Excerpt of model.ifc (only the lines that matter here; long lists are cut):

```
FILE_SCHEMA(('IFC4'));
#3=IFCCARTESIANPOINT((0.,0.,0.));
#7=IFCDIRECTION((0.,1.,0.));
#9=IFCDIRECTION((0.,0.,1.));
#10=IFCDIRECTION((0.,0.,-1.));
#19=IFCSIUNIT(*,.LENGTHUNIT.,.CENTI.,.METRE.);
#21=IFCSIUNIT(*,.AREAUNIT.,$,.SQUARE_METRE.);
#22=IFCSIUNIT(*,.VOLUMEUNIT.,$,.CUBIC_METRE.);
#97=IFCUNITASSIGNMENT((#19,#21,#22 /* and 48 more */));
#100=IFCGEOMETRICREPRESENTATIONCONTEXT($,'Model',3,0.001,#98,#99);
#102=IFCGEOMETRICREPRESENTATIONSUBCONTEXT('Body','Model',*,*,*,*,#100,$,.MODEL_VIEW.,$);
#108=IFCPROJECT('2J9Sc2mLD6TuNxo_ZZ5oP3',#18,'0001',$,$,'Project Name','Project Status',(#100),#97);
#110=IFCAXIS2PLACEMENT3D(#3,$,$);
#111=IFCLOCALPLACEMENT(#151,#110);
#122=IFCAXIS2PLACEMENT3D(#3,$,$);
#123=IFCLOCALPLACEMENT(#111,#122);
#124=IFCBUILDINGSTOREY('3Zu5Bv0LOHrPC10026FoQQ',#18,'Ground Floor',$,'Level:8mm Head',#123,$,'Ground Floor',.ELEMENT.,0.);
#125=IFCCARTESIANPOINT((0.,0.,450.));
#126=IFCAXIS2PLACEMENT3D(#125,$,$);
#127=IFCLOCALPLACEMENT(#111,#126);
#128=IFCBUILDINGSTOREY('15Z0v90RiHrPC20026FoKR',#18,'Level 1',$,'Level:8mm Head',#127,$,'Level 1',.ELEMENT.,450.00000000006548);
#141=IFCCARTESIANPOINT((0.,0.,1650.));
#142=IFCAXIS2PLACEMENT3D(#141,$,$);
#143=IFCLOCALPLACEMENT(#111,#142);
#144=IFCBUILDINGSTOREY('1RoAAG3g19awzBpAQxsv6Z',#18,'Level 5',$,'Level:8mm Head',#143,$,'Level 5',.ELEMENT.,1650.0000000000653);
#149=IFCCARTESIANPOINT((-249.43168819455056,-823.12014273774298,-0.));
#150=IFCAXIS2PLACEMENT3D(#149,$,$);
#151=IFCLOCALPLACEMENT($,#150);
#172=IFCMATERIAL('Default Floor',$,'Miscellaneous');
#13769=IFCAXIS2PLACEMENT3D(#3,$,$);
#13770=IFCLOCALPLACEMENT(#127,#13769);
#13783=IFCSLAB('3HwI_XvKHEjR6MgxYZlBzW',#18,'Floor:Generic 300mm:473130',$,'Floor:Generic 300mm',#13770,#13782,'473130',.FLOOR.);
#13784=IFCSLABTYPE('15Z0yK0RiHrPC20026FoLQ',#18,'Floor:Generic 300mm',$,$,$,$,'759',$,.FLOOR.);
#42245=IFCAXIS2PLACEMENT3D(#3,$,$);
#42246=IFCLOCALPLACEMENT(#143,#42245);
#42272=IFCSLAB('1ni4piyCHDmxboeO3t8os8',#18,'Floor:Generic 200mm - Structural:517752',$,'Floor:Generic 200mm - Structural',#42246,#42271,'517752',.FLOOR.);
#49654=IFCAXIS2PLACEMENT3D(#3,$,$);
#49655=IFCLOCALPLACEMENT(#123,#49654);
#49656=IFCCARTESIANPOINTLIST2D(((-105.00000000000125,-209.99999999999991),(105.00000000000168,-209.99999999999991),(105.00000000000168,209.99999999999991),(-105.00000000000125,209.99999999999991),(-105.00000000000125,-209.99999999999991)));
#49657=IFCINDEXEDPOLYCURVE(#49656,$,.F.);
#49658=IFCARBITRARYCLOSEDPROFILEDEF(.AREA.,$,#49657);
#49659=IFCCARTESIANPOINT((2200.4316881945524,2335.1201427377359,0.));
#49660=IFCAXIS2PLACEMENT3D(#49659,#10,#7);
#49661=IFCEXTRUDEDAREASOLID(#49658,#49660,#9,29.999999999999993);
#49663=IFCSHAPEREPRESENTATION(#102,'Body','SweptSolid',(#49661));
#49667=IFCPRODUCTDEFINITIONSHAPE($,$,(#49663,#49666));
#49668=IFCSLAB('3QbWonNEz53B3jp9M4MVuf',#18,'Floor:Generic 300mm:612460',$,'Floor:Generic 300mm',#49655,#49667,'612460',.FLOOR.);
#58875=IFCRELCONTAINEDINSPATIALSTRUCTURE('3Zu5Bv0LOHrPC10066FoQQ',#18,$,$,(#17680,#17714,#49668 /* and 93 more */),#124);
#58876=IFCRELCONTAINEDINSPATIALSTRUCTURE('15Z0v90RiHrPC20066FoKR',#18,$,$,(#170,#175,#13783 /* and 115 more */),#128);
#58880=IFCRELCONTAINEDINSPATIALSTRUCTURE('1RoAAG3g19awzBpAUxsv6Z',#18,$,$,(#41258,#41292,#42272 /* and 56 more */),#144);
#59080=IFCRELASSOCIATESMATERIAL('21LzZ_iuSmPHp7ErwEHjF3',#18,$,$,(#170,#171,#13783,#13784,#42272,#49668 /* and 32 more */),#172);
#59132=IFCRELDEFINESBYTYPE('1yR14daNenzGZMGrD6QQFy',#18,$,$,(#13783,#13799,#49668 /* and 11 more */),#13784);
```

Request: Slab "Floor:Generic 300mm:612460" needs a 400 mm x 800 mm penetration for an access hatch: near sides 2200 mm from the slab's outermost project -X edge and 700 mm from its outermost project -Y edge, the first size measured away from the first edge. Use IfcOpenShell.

```python
import numpy as np
import ifcopenshell
import ifcopenshell.api.feature
import ifcopenshell.api.geometry
import ifcopenshell.api.root
import ifcopenshell.geom
import ifcopenshell.util.placement
import ifcopenshell.util.representation
import ifcopenshell.util.shape
import ifcopenshell.util.unit

model = ifcopenshell.open("model.ifc")
unit_scale = ifcopenshell.util.unit.calculate_unit_scale(model)
settings = ifcopenshell.geom.settings()


def volume(element):
    """Net volume in cubic metres, openings subtracted."""
    shape = ifcopenshell.geom.create_shape(settings, element)
    return ifcopenshell.util.shape.get_volume(shape.geometry)


slab = model.by_guid("3QbWonNEz53B3jp9M4MVuf")
before = volume(slab)

# Extent in the slab's own axes, in metres. The edges named are its -X and -Y sides.
slab_shape = ifcopenshell.geom.create_shape(settings, slab)
vertices = ifcopenshell.util.shape.get_vertices(slab_shape.geometry)
x_min, y_min, bottom = vertices.min(axis=0)
top = vertices[:, 2].max()

opening = ifcopenshell.api.root.create_entity(model, ifc_class="IfcOpeningElement", name="Access hatch opening", predefined_type="OPENING")
context = ifcopenshell.util.representation.get_context(model, "Model", "Body", "MODEL_VIEW")
width, depth = 0.4, 0.8
outline = [(0.0, 0.0), (width, 0.0), (width, depth), (0.0, depth), (0.0, 0.0)]
# Overshoot both faces by 50 mm so the cut is clean.
shape = ifcopenshell.api.geometry.add_slab_representation(
    model, context=context, depth=top - bottom + 0.1, polyline=outline
)
ifcopenshell.api.geometry.assign_representation(model, product=opening, representation=shape)

matrix = ifcopenshell.util.placement.get_local_placement(slab.ObjectPlacement)
matrix[:, 3] = matrix @ np.append(np.array([x_min + 2.2, y_min + 0.7, bottom - 0.05]) / unit_scale, 1.0)
ifcopenshell.api.geometry.edit_object_placement(model, product=opening, matrix=matrix, is_si=False)
ifcopenshell.api.feature.add_feature(model, feature=opening, element=slab)

after = volume(slab)

print(f"slab volume {before:.3f} -> {after:.3f} m3")

model.write("model_rev.ifc")
```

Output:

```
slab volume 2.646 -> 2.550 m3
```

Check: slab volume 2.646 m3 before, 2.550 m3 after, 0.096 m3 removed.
